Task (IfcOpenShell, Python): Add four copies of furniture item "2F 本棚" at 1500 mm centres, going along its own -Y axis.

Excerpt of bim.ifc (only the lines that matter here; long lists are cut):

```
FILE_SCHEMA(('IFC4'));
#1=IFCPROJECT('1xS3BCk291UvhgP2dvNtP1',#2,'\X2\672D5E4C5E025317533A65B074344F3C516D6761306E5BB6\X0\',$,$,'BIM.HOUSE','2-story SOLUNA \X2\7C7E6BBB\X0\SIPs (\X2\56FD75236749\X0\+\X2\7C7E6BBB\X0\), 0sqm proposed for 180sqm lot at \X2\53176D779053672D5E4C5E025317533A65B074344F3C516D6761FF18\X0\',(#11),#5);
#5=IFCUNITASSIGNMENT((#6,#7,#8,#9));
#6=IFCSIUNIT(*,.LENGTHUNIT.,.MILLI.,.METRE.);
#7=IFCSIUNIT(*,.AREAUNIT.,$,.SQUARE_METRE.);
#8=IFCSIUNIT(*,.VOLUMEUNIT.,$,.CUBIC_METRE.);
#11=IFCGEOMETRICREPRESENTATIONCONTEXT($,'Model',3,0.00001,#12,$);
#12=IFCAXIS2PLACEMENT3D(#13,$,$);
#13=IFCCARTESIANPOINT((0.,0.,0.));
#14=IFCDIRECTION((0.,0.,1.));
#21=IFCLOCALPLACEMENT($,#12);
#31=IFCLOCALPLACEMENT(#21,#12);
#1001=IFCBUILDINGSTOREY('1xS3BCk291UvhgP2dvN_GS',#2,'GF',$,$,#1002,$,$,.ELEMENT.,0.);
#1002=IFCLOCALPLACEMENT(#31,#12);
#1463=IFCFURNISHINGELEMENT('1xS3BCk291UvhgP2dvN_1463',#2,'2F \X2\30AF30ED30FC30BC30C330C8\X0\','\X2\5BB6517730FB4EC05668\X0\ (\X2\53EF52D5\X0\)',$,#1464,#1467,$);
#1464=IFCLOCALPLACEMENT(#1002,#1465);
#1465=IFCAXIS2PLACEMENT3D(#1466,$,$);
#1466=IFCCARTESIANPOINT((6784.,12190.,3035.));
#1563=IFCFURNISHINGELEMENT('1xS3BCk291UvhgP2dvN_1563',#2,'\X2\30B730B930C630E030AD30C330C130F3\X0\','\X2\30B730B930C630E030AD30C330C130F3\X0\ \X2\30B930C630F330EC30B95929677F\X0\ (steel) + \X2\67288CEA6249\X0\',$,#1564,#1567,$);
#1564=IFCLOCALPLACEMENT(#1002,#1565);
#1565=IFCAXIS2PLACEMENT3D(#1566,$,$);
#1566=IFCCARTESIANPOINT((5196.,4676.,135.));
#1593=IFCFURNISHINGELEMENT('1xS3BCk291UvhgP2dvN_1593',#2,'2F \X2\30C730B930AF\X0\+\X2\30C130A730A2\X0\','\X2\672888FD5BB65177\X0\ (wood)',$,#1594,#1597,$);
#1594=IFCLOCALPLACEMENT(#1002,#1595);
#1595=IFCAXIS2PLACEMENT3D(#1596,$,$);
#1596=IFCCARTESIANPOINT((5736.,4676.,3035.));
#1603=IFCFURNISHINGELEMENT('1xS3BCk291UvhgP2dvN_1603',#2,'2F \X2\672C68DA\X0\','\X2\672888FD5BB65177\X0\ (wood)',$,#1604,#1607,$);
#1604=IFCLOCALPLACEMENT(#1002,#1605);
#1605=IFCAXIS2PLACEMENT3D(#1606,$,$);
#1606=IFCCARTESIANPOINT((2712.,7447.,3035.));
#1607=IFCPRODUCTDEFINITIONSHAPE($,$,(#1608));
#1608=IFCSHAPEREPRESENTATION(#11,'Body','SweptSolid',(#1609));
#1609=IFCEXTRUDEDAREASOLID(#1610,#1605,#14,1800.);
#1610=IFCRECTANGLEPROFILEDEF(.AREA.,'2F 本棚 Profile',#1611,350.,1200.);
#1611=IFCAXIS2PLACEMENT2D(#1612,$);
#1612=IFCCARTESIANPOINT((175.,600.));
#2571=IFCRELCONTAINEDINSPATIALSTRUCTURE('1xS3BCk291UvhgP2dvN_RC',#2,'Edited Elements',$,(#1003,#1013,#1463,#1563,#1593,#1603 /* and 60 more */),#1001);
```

```python
import ifcopenshell
import ifcopenshell.api.geometry
import ifcopenshell.api.root
import ifcopenshell.util.element
import ifcopenshell.util.placement

model = ifcopenshell.open("bim.ifc")


def reuse_history(source, copy):
    """copy_class also copies each property set's owner history, people and application; keep the originals."""
    for rel in copy.IsDefinedBy:
        if rel.is_a("IfcRelDefinesByProperties") and (history := rel.RelatingPropertyDefinition.OwnerHistory):
            rel.RelatingPropertyDefinition.OwnerHistory = source.OwnerHistory
            ifcopenshell.util.element.remove_deep2(model, history)


source = model.by_guid("1xS3BCk291UvhgP2dvN_1603")
base = ifcopenshell.util.placement.get_local_placement(source.ObjectPlacement)
step = -base[:3, 1] * 1500.0

for i in range(1, 5):
    copy = ifcopenshell.api.root.copy_class(model, product=source)
    copy.Representation = ifcopenshell.util.element.copy_deep(
        model, source.Representation, exclude=["IfcGeometricRepresentationContext", "IfcRepresentationMap"]
    )
    reuse_history(source, copy)
    matrix = base.copy()
    matrix[:3, 3] += i * step
    print("added at", matrix[:3, 3].round(3) + 0.0)
    ifcopenshell.api.geometry.edit_object_placement(model, product=copy, matrix=matrix, is_si=False)

model.write("bim_edited.ifc")
```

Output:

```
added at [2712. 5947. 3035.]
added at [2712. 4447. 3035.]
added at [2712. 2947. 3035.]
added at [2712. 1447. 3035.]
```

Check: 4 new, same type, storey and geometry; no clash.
